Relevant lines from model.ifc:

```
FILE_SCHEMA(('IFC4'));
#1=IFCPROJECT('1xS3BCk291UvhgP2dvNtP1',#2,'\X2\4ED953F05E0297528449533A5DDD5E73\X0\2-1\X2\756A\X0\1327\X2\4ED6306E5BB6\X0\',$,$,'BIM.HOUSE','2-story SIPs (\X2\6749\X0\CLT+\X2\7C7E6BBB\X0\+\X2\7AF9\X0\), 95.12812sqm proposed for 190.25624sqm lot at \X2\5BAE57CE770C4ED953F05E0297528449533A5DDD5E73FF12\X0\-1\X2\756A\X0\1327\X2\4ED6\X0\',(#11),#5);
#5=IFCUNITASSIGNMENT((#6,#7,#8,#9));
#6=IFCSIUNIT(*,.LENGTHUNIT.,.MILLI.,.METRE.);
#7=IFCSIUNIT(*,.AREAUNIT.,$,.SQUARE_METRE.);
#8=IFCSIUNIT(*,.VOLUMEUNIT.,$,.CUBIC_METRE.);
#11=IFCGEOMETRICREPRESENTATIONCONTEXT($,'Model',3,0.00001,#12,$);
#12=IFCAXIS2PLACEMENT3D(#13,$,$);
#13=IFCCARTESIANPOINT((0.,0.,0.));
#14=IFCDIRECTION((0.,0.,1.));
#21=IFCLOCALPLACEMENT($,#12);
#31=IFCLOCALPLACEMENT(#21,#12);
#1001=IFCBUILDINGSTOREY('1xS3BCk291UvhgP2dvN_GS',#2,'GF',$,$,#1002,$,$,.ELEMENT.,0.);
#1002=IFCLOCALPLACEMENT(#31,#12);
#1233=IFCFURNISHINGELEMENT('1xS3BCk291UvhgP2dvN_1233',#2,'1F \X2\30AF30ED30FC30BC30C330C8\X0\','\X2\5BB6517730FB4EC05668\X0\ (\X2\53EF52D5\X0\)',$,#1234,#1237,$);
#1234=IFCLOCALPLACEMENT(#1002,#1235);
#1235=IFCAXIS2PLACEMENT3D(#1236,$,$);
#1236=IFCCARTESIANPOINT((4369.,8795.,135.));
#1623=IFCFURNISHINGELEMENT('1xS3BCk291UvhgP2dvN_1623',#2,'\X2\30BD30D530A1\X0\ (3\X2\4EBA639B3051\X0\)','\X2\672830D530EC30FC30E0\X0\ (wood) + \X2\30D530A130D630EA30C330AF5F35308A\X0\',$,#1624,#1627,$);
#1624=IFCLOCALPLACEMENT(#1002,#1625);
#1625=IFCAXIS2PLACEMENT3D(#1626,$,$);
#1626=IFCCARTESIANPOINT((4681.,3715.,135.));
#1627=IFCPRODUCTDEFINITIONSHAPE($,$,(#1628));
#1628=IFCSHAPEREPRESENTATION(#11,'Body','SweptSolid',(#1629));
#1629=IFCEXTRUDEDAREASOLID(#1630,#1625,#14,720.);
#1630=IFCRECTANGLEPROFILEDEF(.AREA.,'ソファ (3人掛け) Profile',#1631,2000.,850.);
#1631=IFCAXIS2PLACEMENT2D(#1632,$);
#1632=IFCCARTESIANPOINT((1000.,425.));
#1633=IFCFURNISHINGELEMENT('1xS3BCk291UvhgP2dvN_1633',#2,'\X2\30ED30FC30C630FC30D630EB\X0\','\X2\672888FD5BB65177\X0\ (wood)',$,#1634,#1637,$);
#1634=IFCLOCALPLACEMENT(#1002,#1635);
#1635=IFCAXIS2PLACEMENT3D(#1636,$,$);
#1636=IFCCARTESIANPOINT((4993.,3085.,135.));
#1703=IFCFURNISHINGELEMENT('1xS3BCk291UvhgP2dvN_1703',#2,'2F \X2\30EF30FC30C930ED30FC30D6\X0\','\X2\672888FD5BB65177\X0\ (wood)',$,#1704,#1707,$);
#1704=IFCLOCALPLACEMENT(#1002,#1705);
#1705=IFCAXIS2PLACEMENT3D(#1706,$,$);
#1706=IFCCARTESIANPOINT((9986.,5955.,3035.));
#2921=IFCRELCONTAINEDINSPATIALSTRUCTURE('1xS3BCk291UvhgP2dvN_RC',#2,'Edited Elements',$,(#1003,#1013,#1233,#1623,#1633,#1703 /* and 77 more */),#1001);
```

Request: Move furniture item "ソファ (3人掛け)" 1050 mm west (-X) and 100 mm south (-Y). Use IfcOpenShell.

```python
import ifcopenshell
import ifcopenshell.api.geometry
import ifcopenshell.util.placement
import ifcopenshell.util.unit

model = ifcopenshell.open("model.ifc")
unit_scale = ifcopenshell.util.unit.calculate_unit_scale(model)

item = model.by_guid("1xS3BCk291UvhgP2dvN_1623")
matrix = ifcopenshell.util.placement.get_local_placement(item.ObjectPlacement)
matrix[0, 3] -= 1.05 / unit_scale
matrix[1, 3] -= 0.1 / unit_scale
ifcopenshell.api.geometry.edit_object_placement(model, product=item, matrix=matrix, is_si=False)

print(ifcopenshell.util.placement.get_local_placement(item.ObjectPlacement).round(3) + 0.0)

model.write("model_edited.ifc")
```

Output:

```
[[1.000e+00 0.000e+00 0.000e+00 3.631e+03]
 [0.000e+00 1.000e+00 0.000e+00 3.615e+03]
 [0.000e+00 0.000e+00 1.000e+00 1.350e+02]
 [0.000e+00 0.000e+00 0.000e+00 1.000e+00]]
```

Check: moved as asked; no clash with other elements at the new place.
